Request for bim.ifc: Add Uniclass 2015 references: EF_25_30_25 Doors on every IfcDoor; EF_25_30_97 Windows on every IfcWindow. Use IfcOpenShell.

First a look at what the model holds.

```python
import ifcopenshell

model = ifcopenshell.open("bim.ifc")
print(model.schema)
print("classifications:", [c.Name for c in model.by_type("IfcClassification")])
for ifc_class in ("IfcDoor", "IfcRoof", "IfcStair", "IfcWall", "IfcWindow"):
    print(ifc_class, len(model.by_type(ifc_class)))
```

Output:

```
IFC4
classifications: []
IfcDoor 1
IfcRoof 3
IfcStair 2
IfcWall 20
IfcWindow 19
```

```python
import ifcopenshell
import ifcopenshell.api.classification

model = ifcopenshell.open("bim.ifc")

system = ifcopenshell.api.classification.add_classification(model, classification="Uniclass 2015")

codes = {
    "IfcDoor": ("EF_25_30_25", "Doors"),
    "IfcWindow": ("EF_25_30_97", "Windows"),
}
for ifc_class, (code, name) in codes.items():
    products = model.by_type(ifc_class)
    ifcopenshell.api.classification.add_reference(
        model, products=products, classification=system, identification=code, name=name
    )
    print(code, len(products))

model.write("bim_updated.ifc")
```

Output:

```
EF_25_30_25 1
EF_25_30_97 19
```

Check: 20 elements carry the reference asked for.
